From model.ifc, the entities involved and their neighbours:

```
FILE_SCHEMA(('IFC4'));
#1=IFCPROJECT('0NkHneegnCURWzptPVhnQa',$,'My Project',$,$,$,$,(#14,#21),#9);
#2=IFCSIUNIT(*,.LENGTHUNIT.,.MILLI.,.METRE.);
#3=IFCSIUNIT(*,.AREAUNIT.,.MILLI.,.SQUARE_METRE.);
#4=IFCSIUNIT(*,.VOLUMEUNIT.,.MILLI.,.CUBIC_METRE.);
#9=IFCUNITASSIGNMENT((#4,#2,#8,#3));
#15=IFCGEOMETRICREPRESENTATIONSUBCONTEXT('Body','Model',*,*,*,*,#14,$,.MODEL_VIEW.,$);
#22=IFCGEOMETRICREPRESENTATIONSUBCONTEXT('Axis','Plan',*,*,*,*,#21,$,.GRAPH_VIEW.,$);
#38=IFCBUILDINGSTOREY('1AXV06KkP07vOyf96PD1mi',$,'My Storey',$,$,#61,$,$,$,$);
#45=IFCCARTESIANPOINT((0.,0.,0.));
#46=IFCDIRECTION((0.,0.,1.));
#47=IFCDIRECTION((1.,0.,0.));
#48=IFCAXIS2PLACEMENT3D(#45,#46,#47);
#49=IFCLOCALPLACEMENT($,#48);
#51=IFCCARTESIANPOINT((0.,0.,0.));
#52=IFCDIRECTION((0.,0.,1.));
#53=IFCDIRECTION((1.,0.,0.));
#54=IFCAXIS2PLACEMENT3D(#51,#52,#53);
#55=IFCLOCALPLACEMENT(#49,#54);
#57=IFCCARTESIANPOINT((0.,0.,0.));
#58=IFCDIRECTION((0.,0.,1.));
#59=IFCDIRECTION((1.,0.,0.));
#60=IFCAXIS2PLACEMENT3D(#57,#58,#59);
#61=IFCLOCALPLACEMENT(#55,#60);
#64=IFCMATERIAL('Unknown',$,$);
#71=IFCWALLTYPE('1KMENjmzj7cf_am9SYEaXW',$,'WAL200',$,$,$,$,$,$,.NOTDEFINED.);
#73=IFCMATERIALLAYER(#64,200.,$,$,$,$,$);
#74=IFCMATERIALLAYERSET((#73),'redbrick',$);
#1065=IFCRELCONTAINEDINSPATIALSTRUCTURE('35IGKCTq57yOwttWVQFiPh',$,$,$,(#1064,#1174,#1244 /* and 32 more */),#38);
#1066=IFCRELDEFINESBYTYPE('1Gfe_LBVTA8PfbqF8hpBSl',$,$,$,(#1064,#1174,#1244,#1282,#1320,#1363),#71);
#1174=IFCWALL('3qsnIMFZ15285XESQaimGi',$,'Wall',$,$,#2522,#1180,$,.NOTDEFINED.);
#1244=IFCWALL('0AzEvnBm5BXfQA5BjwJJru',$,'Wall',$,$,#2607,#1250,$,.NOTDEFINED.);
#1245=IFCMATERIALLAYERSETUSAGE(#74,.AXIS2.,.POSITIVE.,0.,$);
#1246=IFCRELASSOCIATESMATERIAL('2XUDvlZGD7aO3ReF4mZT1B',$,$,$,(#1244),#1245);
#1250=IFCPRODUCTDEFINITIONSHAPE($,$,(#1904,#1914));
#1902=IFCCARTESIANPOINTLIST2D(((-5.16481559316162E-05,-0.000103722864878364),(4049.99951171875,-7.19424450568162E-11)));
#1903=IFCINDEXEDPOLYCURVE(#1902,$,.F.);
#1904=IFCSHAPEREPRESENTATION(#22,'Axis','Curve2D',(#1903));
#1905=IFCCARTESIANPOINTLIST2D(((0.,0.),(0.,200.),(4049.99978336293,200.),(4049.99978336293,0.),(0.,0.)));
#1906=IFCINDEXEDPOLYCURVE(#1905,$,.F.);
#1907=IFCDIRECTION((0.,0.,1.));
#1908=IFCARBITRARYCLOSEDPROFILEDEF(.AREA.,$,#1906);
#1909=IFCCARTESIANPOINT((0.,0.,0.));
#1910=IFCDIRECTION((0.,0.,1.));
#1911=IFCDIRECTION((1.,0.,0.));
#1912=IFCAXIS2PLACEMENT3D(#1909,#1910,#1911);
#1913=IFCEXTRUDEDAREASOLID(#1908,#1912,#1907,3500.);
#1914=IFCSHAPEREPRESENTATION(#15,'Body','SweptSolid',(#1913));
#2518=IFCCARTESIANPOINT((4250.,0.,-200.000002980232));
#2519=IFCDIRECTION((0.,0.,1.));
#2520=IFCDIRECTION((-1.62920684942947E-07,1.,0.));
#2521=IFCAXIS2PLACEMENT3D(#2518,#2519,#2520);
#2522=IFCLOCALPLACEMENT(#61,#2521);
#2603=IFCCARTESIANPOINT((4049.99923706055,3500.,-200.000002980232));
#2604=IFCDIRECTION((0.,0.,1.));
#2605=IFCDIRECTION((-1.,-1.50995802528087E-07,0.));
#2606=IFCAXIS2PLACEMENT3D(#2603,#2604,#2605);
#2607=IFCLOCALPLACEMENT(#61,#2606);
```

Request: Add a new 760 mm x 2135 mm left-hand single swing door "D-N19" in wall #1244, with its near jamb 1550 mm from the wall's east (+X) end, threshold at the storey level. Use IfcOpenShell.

```python
import numpy as np
import ifcopenshell
import ifcopenshell.api.feature
import ifcopenshell.api.geometry
import ifcopenshell.api.root
import ifcopenshell.api.spatial
import ifcopenshell.geom
import ifcopenshell.util.element
import ifcopenshell.util.placement
import ifcopenshell.util.representation
import ifcopenshell.util.shape
import ifcopenshell.util.unit

model = ifcopenshell.open("model.ifc")
unit_scale = ifcopenshell.util.unit.calculate_unit_scale(model)
settings = ifcopenshell.geom.settings()


def volume(element):
    """Net volume in cubic metres, openings subtracted."""
    shape = ifcopenshell.geom.create_shape(settings, element)
    return ifcopenshell.util.shape.get_volume(shape.geometry)


wall = model.by_guid("0AzEvnBm5BXfQA5BjwJJru")
storey = ifcopenshell.util.element.get_container(wall, ifc_class="IfcBuildingStorey")
context = ifcopenshell.util.representation.get_context(model, "Model", "Body", "MODEL_VIEW")
before = volume(wall)

width, height, from_end, sill = 0.76, 2.135, 1.55, 0.0  # metres

# The wall runs along its own X axis, and the end named is its -X end.
wall_shape = ifcopenshell.geom.create_shape(settings, wall)
x, y, z = ifcopenshell.util.shape.get_vertices(wall_shape.geometry).T
start = x.min() + from_end
face, thickness = float(y.min()), float(y.max() - y.min())
wall_matrix = ifcopenshell.util.placement.get_local_placement(wall.ObjectPlacement)
level = ifcopenshell.util.placement.get_local_placement(storey.ObjectPlacement)[2, 3]


def in_wall(x, y):
    """Placement at x, y metres in the wall's axes, at sill height."""
    matrix = wall_matrix.copy()
    matrix[:, 3] = wall_matrix @ np.array([x / unit_scale, y / unit_scale, 0.0, 1.0])
    matrix[2, 3] = level + sill / unit_scale
    return matrix


# Opening: a box that overshoots both wall faces by 50 mm.
opening = ifcopenshell.api.root.create_entity(model, ifc_class="IfcOpeningElement", predefined_type="OPENING")
box = ifcopenshell.api.geometry.add_wall_representation(
    model, context=context, length=width, height=height, thickness=thickness + 0.1
)
ifcopenshell.api.geometry.assign_representation(model, product=opening, representation=box)
ifcopenshell.api.geometry.edit_object_placement(model, product=opening, matrix=in_wall(start, face - 0.05), is_si=False)
ifcopenshell.api.feature.add_feature(model, feature=opening, element=wall)

door = ifcopenshell.api.root.create_entity(model, ifc_class="IfcDoor", name="D-N19", predefined_type="DOOR")
door.OverallWidth, door.OverallHeight = width / unit_scale, height / unit_scale
door.OperationType = "SINGLE_SWING_LEFT"
body = ifcopenshell.api.geometry.add_door_representation(
    model,
    context=context,
    overall_width=door.OverallWidth,
    overall_height=door.OverallHeight,
    operation_type="SINGLE_SWING_LEFT",
    lining_properties={"LiningDepth": thickness / unit_scale, "ThresholdDepth": thickness / unit_scale},
)
ifcopenshell.api.geometry.assign_representation(model, product=door, representation=body)
ifcopenshell.api.spatial.assign_container(model, products=[door], relating_structure=storey)
ifcopenshell.api.feature.add_filling(model, opening=opening, element=door)

# The lining spans the wall, so the door starts at the wall face.
ifcopenshell.api.geometry.edit_object_placement(model, product=door, matrix=in_wall(start, face), is_si=False)

after = volume(wall)

print(f"wall volume {before:.3f} -> {after:.3f} m3")

model.write("model_updated.ifc")
```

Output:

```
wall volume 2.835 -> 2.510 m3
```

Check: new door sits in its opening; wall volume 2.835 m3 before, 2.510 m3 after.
